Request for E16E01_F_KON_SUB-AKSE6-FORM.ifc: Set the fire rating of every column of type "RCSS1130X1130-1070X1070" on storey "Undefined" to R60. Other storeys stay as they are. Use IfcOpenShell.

First a look at what the model holds.

```python
import ifcopenshell
import ifcopenshell.util.element

model = ifcopenshell.open("E16E01_F_KON_SUB-AKSE6-FORM.ifc")
print(model.schema)
storey = next(s for s in model.by_type("IfcBuildingStorey") if s.Name == "Undefined")
columns = [e for e in ifcopenshell.util.element.get_decomposition(storey) if e.is_a("IfcColumn")]
seen = {}
for e in columns:
    element_type = ifcopenshell.util.element.get_type(e)
    key = (element_type.Name if element_type != e and element_type else None, ifcopenshell.util.element.get_pset(e, "Pset_ColumnCommon", "FireRating"))
    seen[key] = seen.get(key, 0) + 1
for (name, value), count in sorted(seen.items(), key=str):
    print(count, "x", name, "|", value)
```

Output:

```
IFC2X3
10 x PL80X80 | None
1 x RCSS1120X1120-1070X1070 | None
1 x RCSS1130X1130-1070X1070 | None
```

```python
import ifcopenshell
import ifcopenshell.api.pset
import ifcopenshell.util.element

model = ifcopenshell.open("E16E01_F_KON_SUB-AKSE6-FORM.ifc")

storey = next(s for s in model.by_type("IfcBuildingStorey") if s.Name == "Undefined")
columns = [e for e in ifcopenshell.util.element.get_decomposition(storey) if e.is_a("IfcColumn")]

count = 0
for e in columns:
    element_type = ifcopenshell.util.element.get_type(e)
    if element_type in (None, e) or element_type.Name != "RCSS1130X1130-1070X1070":
        continue
    # add_pset returns the element's existing set when there is one.
    pset = ifcopenshell.api.pset.add_pset(model, product=e, name="Pset_ColumnCommon")
    ifcopenshell.api.pset.edit_pset(model, pset=pset, properties={"FireRating": "R60"})
    count += 1

print(count, "columns updated")

model.write("E16E01_F_KON_SUB-AKSE6-FORM_rev.ifc")
```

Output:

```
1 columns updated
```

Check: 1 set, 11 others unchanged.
